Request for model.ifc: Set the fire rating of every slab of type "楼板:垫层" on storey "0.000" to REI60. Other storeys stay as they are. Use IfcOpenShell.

First a look at what the model holds.

```python
import ifcopenshell
import ifcopenshell.util.element

model = ifcopenshell.open("model.ifc")
print(model.schema)
storey = next(s for s in model.by_type("IfcBuildingStorey") if s.Name == "0.000")
slabs = [e for e in ifcopenshell.util.element.get_decomposition(storey) if e.is_a("IfcSlab")]
seen = {}
for e in slabs:
    element_type = ifcopenshell.util.element.get_type(e)
    key = (element_type.Name if element_type != e and element_type else None, ifcopenshell.util.element.get_pset(e, "Pset_SlabCommon", "FireRating"))
    seen[key] = seen.get(key, 0) + 1
for (name, value), count in sorted(seen.items(), key=str):
    print(count, "x", name, "|", value)
```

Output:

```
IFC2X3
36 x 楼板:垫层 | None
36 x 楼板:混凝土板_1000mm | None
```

```python
import ifcopenshell
import ifcopenshell.api.pset
import ifcopenshell.util.element

model = ifcopenshell.open("model.ifc")

storey = next(s for s in model.by_type("IfcBuildingStorey") if s.Name == "0.000")
slabs = [e for e in ifcopenshell.util.element.get_decomposition(storey) if e.is_a("IfcSlab")]

count = 0
for e in slabs:
    element_type = ifcopenshell.util.element.get_type(e)
    if element_type in (None, e) or element_type.Name != "楼板:垫层":
        continue
    # add_pset returns the element's existing set when there is one.
    pset = ifcopenshell.api.pset.add_pset(model, product=e, name="Pset_SlabCommon")
    ifcopenshell.api.pset.edit_pset(model, pset=pset, properties={"FireRating": "REI60"})
    count += 1

print(count, "slabs updated")

model.write("model_edited.ifc")
```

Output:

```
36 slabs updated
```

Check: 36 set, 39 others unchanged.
